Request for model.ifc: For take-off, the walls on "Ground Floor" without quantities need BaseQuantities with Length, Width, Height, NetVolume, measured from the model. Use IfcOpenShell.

First a look at what the model holds.

```python
import ifcopenshell
import ifcopenshell.util.element
import ifcopenshell.util.unit

model = ifcopenshell.open("model.ifc")
print(model.schema)
for unit_type in ("LENGTHUNIT", "AREAUNIT", "VOLUMEUNIT"):
    print(unit_type, ifcopenshell.util.unit.calculate_unit_scale(model, unit_type))
storey = next(s for s in model.by_type("IfcBuildingStorey") if s.Name == "Ground Floor")
walls = [e for e in ifcopenshell.util.element.get_decomposition(storey) if e.is_a("IfcWall")]
for e in sorted(walls, key=lambda e: e.id()):
    print(e.id(), e.is_a(), e.Name, list(ifcopenshell.util.element.get_psets(e, qtos_only=True)), sep=" | ")
```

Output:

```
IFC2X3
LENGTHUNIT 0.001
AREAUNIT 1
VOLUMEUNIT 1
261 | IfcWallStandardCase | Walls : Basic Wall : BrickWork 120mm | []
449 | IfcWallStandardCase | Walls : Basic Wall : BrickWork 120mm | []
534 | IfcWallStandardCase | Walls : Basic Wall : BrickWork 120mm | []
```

```python
import ifcopenshell
import ifcopenshell.api.pset
import ifcopenshell.geom
import ifcopenshell.util.element
import ifcopenshell.util.shape
import ifcopenshell.util.unit

model = ifcopenshell.open("model.ifc")
unit_scale = ifcopenshell.util.unit.calculate_unit_scale(model)
volume_scale = ifcopenshell.util.unit.calculate_unit_scale(model, "VOLUMEUNIT")
settings = ifcopenshell.geom.settings()

storey = next(s for s in model.by_type("IfcBuildingStorey") if s.Name == "Ground Floor")
walls = [e for e in ifcopenshell.util.element.get_decomposition(storey) if e.is_a("IfcWall")]

for e in sorted(walls, key=lambda e: e.id()):
    if ifcopenshell.util.element.get_psets(e, qtos_only=True, should_inherit=False):
        continue
    # Geometry comes back in metres, in the element's own axes.
    shape = ifcopenshell.geom.create_shape(settings, e)
    values = {
        "Length": ifcopenshell.util.shape.get_x(shape.geometry) / unit_scale,
        "Width": ifcopenshell.util.shape.get_y(shape.geometry) / unit_scale,
        "Height": ifcopenshell.util.shape.get_z(shape.geometry) / unit_scale,
        "NetVolume": ifcopenshell.util.shape.get_volume(shape.geometry) / volume_scale,
    }
    qto = ifcopenshell.api.pset.add_qto(model, product=e, name="BaseQuantities")
    ifcopenshell.api.pset.edit_qto(model, qto=qto, properties=values)
    print(e.id(), {k: round(v, 3) for k, v in values.items()})

model.write("model_updated.ifc")
```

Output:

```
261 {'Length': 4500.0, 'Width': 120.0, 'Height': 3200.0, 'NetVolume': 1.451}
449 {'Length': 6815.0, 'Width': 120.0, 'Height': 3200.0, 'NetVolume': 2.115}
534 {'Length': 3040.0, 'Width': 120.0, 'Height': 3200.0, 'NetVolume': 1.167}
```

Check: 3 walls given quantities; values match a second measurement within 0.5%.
